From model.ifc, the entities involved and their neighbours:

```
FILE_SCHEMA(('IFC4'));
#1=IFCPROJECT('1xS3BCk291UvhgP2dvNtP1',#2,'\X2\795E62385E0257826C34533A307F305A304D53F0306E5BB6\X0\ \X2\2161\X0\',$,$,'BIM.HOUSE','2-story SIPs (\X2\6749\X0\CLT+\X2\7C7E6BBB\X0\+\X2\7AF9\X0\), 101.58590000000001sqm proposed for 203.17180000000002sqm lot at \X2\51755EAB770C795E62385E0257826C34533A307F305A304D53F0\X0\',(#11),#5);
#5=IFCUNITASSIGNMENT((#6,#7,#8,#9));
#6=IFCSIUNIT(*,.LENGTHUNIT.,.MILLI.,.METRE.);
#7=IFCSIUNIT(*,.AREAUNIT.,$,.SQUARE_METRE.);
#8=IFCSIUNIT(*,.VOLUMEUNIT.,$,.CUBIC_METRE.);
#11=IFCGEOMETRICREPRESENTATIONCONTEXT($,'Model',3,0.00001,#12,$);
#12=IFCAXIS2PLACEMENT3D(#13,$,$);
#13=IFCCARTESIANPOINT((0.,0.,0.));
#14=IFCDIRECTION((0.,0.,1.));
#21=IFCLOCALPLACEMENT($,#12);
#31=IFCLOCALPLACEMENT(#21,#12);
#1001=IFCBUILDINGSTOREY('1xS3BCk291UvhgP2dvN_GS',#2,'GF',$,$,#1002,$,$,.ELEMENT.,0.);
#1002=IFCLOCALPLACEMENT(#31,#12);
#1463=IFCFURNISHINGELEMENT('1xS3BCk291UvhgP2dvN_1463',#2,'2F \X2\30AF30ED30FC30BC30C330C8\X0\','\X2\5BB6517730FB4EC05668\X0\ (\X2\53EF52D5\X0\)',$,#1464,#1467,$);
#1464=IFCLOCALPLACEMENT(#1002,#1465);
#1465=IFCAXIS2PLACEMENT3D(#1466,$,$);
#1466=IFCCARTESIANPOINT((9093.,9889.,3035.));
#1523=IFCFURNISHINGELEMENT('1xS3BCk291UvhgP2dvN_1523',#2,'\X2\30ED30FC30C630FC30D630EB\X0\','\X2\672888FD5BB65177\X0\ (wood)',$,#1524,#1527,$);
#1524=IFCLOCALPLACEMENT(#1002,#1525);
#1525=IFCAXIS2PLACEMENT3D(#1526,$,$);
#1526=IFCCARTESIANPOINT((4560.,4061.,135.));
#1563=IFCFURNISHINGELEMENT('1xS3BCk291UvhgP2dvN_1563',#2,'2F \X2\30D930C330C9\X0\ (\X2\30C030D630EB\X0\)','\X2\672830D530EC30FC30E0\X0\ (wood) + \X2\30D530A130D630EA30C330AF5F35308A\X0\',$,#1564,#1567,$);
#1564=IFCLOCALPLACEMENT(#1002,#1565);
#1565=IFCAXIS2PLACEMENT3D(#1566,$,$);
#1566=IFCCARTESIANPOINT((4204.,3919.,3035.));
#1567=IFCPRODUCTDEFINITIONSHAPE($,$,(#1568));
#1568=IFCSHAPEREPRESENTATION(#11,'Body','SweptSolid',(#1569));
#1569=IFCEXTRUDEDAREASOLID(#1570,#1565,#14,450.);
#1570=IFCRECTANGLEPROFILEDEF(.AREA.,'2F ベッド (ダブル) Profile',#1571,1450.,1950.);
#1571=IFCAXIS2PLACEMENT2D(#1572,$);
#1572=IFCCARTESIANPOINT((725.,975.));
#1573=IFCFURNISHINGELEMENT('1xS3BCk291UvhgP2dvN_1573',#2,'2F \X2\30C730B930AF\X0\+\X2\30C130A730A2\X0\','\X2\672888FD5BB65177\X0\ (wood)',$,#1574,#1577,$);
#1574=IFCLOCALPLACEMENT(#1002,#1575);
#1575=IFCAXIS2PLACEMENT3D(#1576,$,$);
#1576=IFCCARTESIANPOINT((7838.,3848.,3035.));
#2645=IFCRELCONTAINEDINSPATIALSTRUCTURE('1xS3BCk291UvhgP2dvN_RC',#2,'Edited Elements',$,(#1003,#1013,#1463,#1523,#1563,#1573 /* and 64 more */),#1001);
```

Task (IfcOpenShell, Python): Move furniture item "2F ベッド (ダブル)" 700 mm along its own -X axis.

```python
import ifcopenshell
import ifcopenshell.api.geometry
import ifcopenshell.util.placement

model = ifcopenshell.open("model.ifc")

item = model.by_guid("1xS3BCk291UvhgP2dvN_1563")
matrix = ifcopenshell.util.placement.get_local_placement(item.ObjectPlacement)
matrix[:3, 3] -= matrix[:3, 0] * 700.0
ifcopenshell.api.geometry.edit_object_placement(model, product=item, matrix=matrix, is_si=False)

print(ifcopenshell.util.placement.get_local_placement(item.ObjectPlacement).round(3) + 0.0)

model.write("model_edited.ifc")
```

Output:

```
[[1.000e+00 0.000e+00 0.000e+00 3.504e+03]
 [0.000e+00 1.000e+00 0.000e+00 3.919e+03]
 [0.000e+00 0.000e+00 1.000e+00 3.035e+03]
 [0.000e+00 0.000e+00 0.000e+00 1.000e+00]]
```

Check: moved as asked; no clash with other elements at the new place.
